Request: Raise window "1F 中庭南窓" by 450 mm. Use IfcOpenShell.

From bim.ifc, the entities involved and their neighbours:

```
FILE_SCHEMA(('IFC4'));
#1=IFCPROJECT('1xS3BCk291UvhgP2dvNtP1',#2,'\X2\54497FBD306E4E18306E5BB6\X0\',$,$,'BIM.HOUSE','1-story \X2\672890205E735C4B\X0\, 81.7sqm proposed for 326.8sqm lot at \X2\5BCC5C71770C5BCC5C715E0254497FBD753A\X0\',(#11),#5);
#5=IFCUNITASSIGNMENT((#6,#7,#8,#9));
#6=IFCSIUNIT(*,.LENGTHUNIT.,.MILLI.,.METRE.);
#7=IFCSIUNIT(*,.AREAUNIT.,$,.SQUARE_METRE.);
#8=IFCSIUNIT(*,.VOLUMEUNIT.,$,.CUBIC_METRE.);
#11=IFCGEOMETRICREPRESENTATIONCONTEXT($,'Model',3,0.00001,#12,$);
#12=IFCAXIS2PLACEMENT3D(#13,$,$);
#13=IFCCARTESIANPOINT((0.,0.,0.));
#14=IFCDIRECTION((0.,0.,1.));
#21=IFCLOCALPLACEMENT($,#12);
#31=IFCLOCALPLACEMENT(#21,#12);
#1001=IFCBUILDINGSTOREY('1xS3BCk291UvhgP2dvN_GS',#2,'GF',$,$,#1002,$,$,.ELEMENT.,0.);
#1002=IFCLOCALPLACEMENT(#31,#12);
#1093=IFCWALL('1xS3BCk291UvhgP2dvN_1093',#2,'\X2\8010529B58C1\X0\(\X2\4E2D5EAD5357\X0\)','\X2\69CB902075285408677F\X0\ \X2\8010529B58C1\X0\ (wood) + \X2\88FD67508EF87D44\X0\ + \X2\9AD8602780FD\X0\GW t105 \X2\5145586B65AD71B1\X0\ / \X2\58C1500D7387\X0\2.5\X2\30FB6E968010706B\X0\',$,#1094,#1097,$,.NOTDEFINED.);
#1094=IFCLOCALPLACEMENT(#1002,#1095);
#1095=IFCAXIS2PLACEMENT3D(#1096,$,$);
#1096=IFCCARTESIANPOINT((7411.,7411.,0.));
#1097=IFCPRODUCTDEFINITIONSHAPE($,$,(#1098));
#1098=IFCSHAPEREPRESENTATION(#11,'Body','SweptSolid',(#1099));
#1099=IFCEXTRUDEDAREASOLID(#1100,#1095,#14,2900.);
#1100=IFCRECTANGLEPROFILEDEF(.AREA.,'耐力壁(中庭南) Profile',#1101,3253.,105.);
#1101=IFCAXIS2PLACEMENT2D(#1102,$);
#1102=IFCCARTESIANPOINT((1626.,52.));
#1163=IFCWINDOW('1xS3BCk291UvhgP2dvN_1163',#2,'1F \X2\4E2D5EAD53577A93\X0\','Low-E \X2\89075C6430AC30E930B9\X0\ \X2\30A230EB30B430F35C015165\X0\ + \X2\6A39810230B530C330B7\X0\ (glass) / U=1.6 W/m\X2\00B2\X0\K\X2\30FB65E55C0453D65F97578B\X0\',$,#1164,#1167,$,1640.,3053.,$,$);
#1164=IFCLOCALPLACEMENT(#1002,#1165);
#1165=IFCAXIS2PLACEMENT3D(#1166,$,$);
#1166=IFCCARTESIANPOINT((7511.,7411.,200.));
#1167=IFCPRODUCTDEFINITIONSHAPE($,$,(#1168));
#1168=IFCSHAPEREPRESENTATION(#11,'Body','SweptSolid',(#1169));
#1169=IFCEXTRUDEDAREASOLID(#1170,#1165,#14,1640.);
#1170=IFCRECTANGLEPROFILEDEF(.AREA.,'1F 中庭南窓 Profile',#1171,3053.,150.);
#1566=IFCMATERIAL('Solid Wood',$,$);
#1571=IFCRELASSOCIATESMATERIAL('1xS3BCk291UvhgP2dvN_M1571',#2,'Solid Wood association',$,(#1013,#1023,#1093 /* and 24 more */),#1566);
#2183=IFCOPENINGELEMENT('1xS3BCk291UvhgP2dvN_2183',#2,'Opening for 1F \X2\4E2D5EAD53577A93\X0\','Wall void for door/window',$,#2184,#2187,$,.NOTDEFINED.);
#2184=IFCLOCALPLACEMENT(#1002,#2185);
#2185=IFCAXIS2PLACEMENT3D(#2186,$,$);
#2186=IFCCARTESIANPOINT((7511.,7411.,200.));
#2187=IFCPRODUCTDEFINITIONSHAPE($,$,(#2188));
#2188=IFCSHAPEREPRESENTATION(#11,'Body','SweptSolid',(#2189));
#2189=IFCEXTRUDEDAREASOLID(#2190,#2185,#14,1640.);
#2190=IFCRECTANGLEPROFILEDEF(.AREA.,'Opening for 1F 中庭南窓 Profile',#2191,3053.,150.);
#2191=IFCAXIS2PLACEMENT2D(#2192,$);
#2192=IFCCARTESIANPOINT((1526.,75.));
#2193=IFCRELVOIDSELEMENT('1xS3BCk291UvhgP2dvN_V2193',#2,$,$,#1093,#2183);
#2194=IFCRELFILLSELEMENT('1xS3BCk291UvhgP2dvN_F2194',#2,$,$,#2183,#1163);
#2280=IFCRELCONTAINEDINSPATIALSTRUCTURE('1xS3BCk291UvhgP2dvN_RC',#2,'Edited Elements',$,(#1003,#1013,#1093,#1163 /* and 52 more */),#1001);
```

```python
import numpy as np
import ifcopenshell
import ifcopenshell.api.geometry
import ifcopenshell.util.placement
import ifcopenshell.util.unit

model = ifcopenshell.open("bim.ifc")
unit_scale = ifcopenshell.util.unit.calculate_unit_scale(model)

window = model.by_id(1163)
opening = window.FillsVoids[0].RelatingOpeningElement
dz = 0.45 / unit_scale

shift = np.array([0.0, 0.0, dz])
# The window is not placed relative to its opening, so move both.
for product in (opening, window):
    matrix = ifcopenshell.util.placement.get_local_placement(product.ObjectPlacement)
    matrix[:3, 3] += shift
    ifcopenshell.api.geometry.edit_object_placement(model, product=product, matrix=matrix, is_si=False)

print(f"moved by {dz * unit_scale:+.3f} m")

model.write("bim_updated.ifc")
```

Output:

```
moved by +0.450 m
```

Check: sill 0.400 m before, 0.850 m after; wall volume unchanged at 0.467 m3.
